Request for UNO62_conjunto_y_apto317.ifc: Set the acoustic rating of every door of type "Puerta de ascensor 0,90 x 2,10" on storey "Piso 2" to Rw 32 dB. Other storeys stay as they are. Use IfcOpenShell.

First a look at what the model holds.

```python
import ifcopenshell
import ifcopenshell.util.element

model = ifcopenshell.open("UNO62_conjunto_y_apto317.ifc")
print(model.schema)
storey = next(s for s in model.by_type("IfcBuildingStorey") if s.Name == "Piso 2")
doors = [e for e in ifcopenshell.util.element.get_decomposition(storey) if e.is_a("IfcDoor")]
seen = {}
for e in doors:
    element_type = ifcopenshell.util.element.get_type(e)
    key = (element_type.Name if element_type != e and element_type else None, ifcopenshell.util.element.get_pset(e, "Pset_DoorCommon", "AcousticRating"))
    seen[key] = seen.get(key, 0) + 1
for (name, value), count in sorted(seen.items(), key=str):
    print(count, "x", name, "|", value)
```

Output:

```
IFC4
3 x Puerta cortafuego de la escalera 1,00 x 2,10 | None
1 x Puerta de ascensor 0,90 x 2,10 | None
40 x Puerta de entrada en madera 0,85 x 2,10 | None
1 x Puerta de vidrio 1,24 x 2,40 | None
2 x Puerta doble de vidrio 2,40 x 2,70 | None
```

```python
import ifcopenshell
import ifcopenshell.api.pset
import ifcopenshell.util.element

model = ifcopenshell.open("UNO62_conjunto_y_apto317.ifc")

storey = next(s for s in model.by_type("IfcBuildingStorey") if s.Name == "Piso 2")
doors = [e for e in ifcopenshell.util.element.get_decomposition(storey) if e.is_a("IfcDoor")]

count = 0
for e in doors:
    element_type = ifcopenshell.util.element.get_type(e)
    if element_type in (None, e) or element_type.Name != "Puerta de ascensor 0,90 x 2,10":
        continue
    found = ifcopenshell.util.element.get_pset(e, "Pset_DoorCommon", should_inherit=False)
    if found:
        pset = model.by_id(found["id"])
        if len(ifcopenshell.util.element.get_elements_by_pset(pset)) > 1:
            pset = ifcopenshell.api.pset.unshare_pset(model, products=[e], pset=pset)[0]
    else:
        pset = ifcopenshell.api.pset.add_pset(model, product=e, name="Pset_DoorCommon")
    ifcopenshell.api.pset.edit_pset(model, pset=pset, properties={"AcousticRating": "Rw 32 dB"})
    count += 1

print(count, "doors updated")

model.write("UNO62_conjunto_y_apto317-out.ifc")
```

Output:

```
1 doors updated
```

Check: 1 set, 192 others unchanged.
